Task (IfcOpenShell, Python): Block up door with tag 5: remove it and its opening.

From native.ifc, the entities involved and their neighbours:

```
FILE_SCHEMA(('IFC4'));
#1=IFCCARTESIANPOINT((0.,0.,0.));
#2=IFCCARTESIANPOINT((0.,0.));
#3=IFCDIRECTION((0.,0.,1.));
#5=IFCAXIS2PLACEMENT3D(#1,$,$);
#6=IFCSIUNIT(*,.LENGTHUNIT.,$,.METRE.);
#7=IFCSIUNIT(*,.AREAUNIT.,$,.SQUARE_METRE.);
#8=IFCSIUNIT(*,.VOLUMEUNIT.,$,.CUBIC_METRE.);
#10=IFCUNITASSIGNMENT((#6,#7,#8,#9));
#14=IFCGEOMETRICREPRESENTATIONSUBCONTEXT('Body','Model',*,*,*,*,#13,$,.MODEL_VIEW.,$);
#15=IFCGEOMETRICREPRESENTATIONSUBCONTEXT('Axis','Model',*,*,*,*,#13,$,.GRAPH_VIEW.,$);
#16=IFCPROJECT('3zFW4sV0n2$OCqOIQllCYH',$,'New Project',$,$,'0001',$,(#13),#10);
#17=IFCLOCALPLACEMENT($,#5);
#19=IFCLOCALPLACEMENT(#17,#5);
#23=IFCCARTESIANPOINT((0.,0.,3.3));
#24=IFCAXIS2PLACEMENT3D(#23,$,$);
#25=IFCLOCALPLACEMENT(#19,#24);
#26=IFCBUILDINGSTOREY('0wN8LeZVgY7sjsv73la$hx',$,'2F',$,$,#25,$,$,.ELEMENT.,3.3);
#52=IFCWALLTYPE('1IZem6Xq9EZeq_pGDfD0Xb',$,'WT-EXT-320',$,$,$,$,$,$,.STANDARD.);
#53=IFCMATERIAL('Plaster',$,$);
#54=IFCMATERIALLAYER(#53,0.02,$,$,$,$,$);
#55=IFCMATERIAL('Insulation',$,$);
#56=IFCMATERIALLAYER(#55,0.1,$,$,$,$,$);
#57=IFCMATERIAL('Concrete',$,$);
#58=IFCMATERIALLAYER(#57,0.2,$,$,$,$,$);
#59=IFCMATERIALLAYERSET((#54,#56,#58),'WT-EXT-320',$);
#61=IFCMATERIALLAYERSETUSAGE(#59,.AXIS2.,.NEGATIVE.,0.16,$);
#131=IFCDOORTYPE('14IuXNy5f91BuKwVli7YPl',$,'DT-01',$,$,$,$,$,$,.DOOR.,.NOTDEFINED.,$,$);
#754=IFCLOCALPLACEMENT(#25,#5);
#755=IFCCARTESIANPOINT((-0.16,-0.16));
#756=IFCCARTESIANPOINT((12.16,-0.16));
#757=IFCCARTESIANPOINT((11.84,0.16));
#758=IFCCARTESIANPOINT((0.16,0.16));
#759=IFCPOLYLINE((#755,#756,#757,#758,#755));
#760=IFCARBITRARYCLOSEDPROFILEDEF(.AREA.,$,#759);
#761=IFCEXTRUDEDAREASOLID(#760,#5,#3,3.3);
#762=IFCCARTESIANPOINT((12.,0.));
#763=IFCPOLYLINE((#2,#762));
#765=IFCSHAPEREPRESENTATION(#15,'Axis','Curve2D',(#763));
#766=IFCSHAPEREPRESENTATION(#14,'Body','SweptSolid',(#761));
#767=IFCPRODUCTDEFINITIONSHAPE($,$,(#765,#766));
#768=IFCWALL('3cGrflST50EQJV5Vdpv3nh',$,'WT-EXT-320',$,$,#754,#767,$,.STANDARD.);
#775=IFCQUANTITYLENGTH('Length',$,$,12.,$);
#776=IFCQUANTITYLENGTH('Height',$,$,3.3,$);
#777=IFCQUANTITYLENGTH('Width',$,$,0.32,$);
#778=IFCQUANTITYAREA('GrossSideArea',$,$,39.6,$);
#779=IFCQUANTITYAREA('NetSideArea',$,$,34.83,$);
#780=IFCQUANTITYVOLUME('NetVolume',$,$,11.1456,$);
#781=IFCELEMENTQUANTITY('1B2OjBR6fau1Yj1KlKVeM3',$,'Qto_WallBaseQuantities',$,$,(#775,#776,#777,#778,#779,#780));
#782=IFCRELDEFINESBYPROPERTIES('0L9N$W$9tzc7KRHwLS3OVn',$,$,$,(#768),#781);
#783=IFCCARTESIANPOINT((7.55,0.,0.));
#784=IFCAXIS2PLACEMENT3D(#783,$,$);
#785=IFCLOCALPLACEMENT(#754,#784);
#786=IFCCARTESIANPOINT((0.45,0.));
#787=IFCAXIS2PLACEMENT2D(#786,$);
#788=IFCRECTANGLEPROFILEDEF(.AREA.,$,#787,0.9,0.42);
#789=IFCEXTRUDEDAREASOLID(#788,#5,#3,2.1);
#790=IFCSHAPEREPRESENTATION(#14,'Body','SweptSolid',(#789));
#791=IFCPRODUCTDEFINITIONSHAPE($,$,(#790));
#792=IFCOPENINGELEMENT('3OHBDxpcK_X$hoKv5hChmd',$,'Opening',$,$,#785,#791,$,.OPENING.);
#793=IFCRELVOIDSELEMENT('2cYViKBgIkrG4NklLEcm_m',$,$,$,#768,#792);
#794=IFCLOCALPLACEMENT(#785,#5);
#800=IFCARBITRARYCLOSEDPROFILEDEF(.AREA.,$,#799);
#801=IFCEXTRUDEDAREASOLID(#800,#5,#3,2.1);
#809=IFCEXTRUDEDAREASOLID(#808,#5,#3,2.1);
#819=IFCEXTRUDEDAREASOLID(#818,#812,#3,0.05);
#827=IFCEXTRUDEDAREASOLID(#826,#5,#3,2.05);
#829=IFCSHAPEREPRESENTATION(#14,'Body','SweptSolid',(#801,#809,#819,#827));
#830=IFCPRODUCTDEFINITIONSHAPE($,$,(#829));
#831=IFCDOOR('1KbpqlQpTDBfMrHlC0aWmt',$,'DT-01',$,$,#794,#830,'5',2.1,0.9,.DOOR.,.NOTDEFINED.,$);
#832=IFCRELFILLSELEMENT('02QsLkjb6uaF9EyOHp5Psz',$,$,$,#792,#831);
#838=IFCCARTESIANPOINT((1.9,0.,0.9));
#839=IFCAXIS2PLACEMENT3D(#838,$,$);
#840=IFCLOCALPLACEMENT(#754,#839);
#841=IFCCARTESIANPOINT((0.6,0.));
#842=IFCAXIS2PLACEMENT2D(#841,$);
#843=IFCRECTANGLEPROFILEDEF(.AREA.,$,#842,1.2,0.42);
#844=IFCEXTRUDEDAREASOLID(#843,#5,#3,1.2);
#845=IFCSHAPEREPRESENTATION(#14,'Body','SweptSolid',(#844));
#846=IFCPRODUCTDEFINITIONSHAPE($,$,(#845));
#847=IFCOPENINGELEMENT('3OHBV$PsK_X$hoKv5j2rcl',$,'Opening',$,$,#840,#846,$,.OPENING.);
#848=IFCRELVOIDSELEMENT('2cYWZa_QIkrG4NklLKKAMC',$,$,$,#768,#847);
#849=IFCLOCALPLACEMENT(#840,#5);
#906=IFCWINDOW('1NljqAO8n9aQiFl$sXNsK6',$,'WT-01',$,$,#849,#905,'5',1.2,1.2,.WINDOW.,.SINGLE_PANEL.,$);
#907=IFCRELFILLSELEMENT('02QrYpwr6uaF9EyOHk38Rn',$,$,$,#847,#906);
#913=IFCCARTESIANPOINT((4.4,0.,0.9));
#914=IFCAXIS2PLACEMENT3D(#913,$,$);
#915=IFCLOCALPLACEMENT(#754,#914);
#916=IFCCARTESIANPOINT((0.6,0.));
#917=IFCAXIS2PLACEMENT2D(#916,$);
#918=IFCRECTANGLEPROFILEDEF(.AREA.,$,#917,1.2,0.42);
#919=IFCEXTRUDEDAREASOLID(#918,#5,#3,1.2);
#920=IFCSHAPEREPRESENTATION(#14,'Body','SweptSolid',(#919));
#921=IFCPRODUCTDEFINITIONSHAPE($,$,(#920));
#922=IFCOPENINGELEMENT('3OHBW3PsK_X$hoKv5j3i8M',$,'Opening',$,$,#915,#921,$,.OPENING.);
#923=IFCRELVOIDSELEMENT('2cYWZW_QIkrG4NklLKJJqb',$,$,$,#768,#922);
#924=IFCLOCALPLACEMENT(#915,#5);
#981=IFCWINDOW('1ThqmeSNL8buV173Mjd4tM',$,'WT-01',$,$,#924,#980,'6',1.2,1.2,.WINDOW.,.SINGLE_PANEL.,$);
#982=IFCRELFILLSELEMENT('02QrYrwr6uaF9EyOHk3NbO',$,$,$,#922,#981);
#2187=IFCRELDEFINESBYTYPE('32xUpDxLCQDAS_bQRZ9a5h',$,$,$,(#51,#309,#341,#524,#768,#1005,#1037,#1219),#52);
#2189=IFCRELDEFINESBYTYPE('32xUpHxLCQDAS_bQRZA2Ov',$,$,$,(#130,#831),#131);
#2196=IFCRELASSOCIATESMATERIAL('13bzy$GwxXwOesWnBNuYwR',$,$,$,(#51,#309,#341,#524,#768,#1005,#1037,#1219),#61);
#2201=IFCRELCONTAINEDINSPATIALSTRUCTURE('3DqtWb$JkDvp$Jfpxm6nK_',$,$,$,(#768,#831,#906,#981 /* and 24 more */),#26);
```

```python
import ifcopenshell
import ifcopenshell.api.feature
import ifcopenshell.api.pset
import ifcopenshell.api.root
import ifcopenshell.geom
import ifcopenshell.util.element
import ifcopenshell.util.shape
import ifcopenshell.util.unit

model = ifcopenshell.open("native.ifc")
area_scale = ifcopenshell.util.unit.calculate_unit_scale(model, "AREAUNIT")
volume_scale = ifcopenshell.util.unit.calculate_unit_scale(model, "VOLUMEUNIT")
settings = ifcopenshell.geom.settings()


def volume(element):
    """Net volume in cubic metres, openings subtracted."""
    shape = ifcopenshell.geom.create_shape(settings, element)
    return ifcopenshell.util.shape.get_volume(shape.geometry)


door = model.by_guid("1KbpqlQpTDBfMrHlC0aWmt")
opening = door.FillsVoids[0].RelatingOpeningElement
wall = opening.VoidsElements[0].RelatingBuildingElement
before = volume(wall)

ifcopenshell.api.root.remove_product(model, product=door)
ifcopenshell.api.feature.remove_feature(model, feature=opening)

after = volume(wall)
thickness = 0.32  # wall thickness in metres

# Update the wall's stored quantities.
qto = model.by_id(ifcopenshell.util.element.get_pset(wall, "Qto_WallBaseQuantities", should_inherit=False)["id"])
ifcopenshell.api.pset.edit_qto(model, qto=qto, properties={
    "NetSideArea": after / thickness / area_scale,
    "NetVolume": after / volume_scale,
})

print(f"wall volume {before:.3f} -> {after:.3f} m3")

model.write("native_updated.ifc")
```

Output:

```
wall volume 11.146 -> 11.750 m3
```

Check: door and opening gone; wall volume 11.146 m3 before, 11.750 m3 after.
